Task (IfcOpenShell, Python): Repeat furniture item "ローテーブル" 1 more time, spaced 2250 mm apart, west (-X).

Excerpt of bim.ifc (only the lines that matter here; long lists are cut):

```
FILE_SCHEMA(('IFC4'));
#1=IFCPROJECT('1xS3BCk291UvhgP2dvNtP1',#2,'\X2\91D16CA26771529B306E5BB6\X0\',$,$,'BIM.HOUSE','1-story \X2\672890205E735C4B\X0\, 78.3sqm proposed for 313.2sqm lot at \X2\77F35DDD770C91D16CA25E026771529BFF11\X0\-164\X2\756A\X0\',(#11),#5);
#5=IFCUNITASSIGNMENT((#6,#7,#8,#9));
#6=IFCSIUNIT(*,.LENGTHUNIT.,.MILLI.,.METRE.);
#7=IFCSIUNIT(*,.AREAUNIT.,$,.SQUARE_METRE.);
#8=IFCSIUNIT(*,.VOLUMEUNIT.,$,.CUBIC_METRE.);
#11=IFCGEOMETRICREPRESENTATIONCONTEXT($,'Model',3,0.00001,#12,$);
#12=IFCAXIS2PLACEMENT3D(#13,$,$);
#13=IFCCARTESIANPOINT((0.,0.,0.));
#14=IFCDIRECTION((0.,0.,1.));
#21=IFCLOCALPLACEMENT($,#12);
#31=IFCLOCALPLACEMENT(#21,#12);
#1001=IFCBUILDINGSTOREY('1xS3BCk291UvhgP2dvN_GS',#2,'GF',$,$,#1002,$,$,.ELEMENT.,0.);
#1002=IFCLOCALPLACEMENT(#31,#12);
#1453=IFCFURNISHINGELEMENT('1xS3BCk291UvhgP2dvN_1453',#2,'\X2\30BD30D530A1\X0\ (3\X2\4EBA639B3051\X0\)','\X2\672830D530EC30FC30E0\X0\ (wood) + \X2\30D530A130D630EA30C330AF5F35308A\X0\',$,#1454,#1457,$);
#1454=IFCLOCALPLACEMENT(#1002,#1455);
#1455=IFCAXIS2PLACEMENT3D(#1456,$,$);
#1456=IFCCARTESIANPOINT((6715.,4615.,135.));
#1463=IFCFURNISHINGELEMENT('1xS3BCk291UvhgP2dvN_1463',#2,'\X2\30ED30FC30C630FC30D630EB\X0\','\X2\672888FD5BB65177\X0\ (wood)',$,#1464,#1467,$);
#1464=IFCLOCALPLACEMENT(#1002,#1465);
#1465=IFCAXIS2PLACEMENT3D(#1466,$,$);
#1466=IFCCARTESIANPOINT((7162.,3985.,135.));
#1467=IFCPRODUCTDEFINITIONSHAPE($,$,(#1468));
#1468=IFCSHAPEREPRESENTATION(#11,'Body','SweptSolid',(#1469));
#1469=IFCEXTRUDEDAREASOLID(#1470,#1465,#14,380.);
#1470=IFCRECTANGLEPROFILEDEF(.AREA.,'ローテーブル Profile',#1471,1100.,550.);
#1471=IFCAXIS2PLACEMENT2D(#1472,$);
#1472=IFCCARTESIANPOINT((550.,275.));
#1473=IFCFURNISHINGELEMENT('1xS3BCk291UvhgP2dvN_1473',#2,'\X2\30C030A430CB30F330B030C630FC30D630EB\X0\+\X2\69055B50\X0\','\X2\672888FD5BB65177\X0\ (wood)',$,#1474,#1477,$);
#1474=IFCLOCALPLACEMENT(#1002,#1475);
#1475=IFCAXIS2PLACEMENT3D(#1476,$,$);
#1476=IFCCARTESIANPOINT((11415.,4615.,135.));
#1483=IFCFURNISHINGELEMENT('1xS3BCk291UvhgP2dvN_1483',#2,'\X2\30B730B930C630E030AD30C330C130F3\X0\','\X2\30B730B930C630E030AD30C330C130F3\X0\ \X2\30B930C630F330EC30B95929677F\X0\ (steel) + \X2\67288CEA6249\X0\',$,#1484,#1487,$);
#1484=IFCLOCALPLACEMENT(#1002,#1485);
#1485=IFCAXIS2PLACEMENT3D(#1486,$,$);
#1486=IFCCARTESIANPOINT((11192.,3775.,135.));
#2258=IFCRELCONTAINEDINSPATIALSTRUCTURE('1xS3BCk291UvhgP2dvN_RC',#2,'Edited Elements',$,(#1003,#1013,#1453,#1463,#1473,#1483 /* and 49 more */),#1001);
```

```python
import numpy as np
import ifcopenshell
import ifcopenshell.api.geometry
import ifcopenshell.api.root
import ifcopenshell.util.element
import ifcopenshell.util.placement
import ifcopenshell.util.unit

model = ifcopenshell.open("bim.ifc")
unit_scale = ifcopenshell.util.unit.calculate_unit_scale(model)


def reuse_history(source, copy):
    """copy_class also copies each property set's owner history, people and application; keep the originals."""
    for rel in copy.IsDefinedBy:
        if rel.is_a("IfcRelDefinesByProperties") and (history := rel.RelatingPropertyDefinition.OwnerHistory):
            rel.RelatingPropertyDefinition.OwnerHistory = source.OwnerHistory
            ifcopenshell.util.element.remove_deep2(model, history)


source = model.by_guid("1xS3BCk291UvhgP2dvN_1463")
base = ifcopenshell.util.placement.get_local_placement(source.ObjectPlacement)
step = np.array([-1.0, 0.0, 0.0]) * 2.25 / unit_scale

for i in range(1, 2):
    copy = ifcopenshell.api.root.copy_class(model, product=source)
    copy.Representation = ifcopenshell.util.element.copy_deep(
        model, source.Representation, exclude=["IfcGeometricRepresentationContext", "IfcRepresentationMap"]
    )
    reuse_history(source, copy)
    matrix = base.copy()
    matrix[:3, 3] += i * step
    print("added at", matrix[:3, 3].round(3) + 0.0)
    ifcopenshell.api.geometry.edit_object_placement(model, product=copy, matrix=matrix, is_si=False)

model.write("bim_v2.ifc")
```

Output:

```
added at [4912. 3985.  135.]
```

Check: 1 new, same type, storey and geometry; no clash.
